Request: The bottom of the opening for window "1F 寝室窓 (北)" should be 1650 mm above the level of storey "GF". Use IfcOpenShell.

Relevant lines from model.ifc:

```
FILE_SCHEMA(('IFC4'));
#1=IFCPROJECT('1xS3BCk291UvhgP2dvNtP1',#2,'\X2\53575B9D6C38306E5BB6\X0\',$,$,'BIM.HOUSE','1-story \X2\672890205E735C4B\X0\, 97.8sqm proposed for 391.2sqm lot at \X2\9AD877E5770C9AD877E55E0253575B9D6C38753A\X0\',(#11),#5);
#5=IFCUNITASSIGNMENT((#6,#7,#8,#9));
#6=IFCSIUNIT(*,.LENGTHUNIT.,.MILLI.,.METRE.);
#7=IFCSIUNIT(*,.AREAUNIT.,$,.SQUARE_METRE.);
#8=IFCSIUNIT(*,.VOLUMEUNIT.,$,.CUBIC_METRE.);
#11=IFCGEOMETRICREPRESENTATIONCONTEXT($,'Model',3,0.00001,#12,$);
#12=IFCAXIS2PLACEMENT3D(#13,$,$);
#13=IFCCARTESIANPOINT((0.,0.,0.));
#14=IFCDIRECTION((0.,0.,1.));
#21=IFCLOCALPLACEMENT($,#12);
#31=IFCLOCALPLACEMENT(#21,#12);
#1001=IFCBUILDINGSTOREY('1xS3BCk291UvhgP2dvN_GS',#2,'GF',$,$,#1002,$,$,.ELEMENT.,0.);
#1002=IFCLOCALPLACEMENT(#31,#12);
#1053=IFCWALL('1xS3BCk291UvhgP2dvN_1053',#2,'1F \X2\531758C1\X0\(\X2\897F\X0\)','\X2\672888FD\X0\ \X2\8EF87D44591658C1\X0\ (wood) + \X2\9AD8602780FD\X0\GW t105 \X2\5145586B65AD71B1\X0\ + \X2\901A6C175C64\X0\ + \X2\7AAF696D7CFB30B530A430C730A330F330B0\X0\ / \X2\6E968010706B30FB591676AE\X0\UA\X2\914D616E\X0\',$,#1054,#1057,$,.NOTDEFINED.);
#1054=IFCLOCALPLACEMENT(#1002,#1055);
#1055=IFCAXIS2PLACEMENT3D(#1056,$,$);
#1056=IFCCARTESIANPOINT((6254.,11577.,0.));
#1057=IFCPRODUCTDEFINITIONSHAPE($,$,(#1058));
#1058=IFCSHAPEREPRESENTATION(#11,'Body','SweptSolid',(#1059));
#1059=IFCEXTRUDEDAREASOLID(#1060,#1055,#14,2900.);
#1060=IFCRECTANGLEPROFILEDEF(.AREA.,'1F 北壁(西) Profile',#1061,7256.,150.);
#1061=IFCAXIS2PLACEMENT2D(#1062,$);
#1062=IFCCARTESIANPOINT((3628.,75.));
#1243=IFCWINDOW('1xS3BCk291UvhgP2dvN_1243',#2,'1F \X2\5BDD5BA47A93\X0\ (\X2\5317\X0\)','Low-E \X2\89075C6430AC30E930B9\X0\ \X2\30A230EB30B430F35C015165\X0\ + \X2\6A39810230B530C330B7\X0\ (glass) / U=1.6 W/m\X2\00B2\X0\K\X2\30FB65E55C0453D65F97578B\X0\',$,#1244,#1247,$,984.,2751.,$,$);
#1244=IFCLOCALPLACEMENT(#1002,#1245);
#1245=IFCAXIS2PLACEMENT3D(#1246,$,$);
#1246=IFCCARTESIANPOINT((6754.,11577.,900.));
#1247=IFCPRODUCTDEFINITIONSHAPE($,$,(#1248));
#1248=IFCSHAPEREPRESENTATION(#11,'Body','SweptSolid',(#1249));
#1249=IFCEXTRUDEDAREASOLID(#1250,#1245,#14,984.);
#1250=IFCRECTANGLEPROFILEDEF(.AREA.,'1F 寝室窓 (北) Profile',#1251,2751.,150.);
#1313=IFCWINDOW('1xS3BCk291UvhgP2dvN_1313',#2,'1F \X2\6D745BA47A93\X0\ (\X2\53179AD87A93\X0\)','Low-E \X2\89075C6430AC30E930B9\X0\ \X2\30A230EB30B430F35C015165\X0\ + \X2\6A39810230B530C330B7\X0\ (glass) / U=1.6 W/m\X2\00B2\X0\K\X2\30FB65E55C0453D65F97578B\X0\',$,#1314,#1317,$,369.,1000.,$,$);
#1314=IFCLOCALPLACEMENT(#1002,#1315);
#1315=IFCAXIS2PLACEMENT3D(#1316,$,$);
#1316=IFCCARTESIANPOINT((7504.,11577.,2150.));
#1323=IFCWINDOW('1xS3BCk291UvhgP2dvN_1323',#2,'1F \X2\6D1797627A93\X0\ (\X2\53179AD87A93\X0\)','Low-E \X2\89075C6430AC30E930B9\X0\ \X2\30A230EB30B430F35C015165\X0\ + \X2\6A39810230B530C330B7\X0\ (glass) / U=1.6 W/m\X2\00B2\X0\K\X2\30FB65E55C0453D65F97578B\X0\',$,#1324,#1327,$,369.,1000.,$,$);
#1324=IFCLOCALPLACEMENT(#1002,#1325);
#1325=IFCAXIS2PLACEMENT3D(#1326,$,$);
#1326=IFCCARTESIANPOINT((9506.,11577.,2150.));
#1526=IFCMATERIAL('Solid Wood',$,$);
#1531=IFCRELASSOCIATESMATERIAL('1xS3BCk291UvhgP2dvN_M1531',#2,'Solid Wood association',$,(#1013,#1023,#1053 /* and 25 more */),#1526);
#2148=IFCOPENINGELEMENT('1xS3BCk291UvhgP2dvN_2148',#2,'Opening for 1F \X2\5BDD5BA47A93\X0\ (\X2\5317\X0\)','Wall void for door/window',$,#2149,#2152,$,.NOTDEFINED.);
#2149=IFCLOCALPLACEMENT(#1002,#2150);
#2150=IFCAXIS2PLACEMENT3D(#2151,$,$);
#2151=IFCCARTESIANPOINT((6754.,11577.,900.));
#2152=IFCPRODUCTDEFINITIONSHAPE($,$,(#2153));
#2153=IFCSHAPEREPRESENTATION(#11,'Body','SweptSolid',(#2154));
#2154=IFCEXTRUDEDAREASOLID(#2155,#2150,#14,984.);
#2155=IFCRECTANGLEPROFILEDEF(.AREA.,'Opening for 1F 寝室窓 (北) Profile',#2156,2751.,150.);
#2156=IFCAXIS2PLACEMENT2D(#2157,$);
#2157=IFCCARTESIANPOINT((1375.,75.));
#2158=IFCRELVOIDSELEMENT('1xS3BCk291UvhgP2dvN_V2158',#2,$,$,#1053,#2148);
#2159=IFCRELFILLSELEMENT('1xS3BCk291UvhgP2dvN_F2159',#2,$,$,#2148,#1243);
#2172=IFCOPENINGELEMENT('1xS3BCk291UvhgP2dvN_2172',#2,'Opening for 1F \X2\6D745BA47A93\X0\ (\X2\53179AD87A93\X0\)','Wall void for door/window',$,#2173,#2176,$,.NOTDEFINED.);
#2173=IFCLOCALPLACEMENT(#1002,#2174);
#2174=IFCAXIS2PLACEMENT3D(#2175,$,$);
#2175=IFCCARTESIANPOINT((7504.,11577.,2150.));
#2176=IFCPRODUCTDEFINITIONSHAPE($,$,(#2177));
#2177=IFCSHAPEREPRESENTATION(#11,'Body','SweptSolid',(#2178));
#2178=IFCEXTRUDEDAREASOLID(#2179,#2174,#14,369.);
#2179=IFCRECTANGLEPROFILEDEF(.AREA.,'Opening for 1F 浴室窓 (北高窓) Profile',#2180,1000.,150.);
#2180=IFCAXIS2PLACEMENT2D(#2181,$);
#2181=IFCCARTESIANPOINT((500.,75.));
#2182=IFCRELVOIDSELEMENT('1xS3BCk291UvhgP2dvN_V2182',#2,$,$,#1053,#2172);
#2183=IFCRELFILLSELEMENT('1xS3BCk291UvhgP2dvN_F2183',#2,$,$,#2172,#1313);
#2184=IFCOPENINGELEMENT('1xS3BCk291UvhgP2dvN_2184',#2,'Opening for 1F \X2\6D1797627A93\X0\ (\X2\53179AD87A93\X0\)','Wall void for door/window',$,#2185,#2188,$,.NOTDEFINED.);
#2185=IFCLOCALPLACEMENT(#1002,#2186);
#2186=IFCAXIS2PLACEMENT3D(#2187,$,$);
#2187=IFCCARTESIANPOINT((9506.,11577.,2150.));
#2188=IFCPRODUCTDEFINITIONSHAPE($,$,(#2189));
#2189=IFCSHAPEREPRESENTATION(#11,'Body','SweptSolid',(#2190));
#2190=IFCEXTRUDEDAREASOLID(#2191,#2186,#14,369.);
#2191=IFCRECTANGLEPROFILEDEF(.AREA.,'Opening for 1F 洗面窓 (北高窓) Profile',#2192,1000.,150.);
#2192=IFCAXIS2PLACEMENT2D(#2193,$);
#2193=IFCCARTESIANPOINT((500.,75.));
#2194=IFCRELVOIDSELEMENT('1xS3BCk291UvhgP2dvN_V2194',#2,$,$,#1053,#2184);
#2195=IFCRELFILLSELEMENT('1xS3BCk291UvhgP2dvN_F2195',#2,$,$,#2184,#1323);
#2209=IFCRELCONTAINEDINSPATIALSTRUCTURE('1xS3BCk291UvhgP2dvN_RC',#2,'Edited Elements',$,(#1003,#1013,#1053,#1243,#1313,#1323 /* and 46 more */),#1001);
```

```python
import numpy as np
import ifcopenshell
import ifcopenshell.api.geometry
import ifcopenshell.geom
import ifcopenshell.util.element
import ifcopenshell.util.placement
import ifcopenshell.util.shape
import ifcopenshell.util.unit

model = ifcopenshell.open("model.ifc")
unit_scale = ifcopenshell.util.unit.calculate_unit_scale(model)

window = model.by_guid("1xS3BCk291UvhgP2dvN_1243")
opening = window.FillsVoids[0].RelatingOpeningElement
storey = ifcopenshell.util.element.get_container(window, ifc_class="IfcBuildingStorey")
level = ifcopenshell.util.placement.get_local_placement(storey.ObjectPlacement)[2, 3]

# The opening's origin need not be at the sill, so measure its lowest point.
shape = ifcopenshell.geom.create_shape(ifcopenshell.geom.settings(), opening)
bottom = ifcopenshell.util.shape.get_shape_bottom_elevation(shape, shape.geometry) / unit_scale
dz = level + 1650.0 - bottom

shift = np.array([0.0, 0.0, dz])
# The window is not placed relative to its opening, so move both.
for product in (opening, window):
    matrix = ifcopenshell.util.placement.get_local_placement(product.ObjectPlacement)
    matrix[:3, 3] += shift
    ifcopenshell.api.geometry.edit_object_placement(model, product=product, matrix=matrix, is_si=False)

print(f"moved by {dz * unit_scale:+.3f} m")

model.write("model_rev.ifc")
```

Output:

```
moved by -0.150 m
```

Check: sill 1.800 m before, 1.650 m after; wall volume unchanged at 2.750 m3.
